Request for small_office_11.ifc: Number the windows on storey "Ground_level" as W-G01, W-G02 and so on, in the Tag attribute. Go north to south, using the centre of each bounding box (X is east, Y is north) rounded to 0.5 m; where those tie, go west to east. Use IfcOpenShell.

First a look at what the model holds.

```python
import ifcopenshell
import ifcopenshell.util.element
import ifcopenshell.util.placement

model = ifcopenshell.open("small_office_11.ifc")
print(model.schema)
storey = next(s for s in model.by_type("IfcBuildingStorey") if s.Name == "Ground_level")
windows = [e for e in ifcopenshell.util.element.get_decomposition(storey) if e.is_a("IfcWindow")]
for e in sorted(windows, key=lambda e: e.id()):
    origin = ifcopenshell.util.placement.get_local_placement(e.ObjectPlacement)[:3, 3]
    print(e.id(), e.Tag, e.Name, origin.round(2) + 0.0, sep=" | ")
```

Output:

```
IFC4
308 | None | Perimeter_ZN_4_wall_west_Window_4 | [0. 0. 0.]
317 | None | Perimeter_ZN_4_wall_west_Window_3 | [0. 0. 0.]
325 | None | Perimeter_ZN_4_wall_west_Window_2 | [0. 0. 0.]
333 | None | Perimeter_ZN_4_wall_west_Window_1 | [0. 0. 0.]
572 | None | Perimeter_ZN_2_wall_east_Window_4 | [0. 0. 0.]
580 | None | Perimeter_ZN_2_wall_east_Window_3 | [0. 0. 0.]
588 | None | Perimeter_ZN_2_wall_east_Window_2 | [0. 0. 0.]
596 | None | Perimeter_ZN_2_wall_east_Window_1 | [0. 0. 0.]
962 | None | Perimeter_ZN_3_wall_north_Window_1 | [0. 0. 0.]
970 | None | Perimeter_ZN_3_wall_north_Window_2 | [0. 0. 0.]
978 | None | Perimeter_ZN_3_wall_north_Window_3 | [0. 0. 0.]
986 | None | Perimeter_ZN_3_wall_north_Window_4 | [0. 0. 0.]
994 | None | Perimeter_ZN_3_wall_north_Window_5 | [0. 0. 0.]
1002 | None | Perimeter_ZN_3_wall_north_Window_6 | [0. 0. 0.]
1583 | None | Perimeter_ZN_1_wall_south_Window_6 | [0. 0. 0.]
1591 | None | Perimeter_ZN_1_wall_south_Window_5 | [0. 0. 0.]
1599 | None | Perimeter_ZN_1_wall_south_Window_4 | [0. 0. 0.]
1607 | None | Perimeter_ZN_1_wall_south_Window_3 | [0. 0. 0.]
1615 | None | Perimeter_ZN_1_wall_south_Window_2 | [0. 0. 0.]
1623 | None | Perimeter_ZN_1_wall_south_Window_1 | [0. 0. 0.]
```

```python
import ifcopenshell
import ifcopenshell.geom
import ifcopenshell.util.element
import ifcopenshell.util.shape

model = ifcopenshell.open("small_office_11.ifc")
settings = ifcopenshell.geom.settings()
settings.set("use-world-coords", True)


def centre(element):
    shape = ifcopenshell.geom.create_shape(settings, element)
    return ifcopenshell.util.shape.get_bbox_centroid(shape.geometry)


storey = next(s for s in model.by_type("IfcBuildingStorey") if s.Name == "Ground_level")
windows = [e for e in ifcopenshell.util.element.get_decomposition(storey) if e.is_a("IfcWindow")]

# Insertion points can sit at a corner or the storey origin, so sort by the geometry (in metres).
centres = {e: centre(e) for e in windows}
windows.sort(key=lambda e: (-round(centres[e][1] / 0.5), centres[e][0]))

for i, e in enumerate(windows, start=1):
    number = f"W-G{i:02d}"
    e.Tag = number
    print(e.id(), number)

model.write("small_office_11-out.ifc")
```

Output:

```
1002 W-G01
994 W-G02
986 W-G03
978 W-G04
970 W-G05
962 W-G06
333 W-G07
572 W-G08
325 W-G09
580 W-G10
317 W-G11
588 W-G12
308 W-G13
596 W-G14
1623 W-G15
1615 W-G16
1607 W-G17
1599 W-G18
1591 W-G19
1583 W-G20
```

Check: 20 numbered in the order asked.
